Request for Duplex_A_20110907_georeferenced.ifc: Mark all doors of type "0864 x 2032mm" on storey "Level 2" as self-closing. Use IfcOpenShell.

First a look at what the model holds.

```python
import ifcopenshell
import ifcopenshell.util.element

model = ifcopenshell.open("Duplex_A_20110907_georeferenced.ifc")
print(model.schema)
storey = next(s for s in model.by_type("IfcBuildingStorey") if s.Name == "Level 2")
doors = [e for e in ifcopenshell.util.element.get_decomposition(storey) if e.is_a("IfcDoor")]
seen = {}
for e in doors:
    element_type = ifcopenshell.util.element.get_type(e)
    key = (element_type.Name if element_type != e and element_type else None, ifcopenshell.util.element.get_pset(e, "Pset_DoorCommon", "SelfClosing"))
    seen[key] = seen.get(key, 0) + 1
for (name, value), count in sorted(seen.items(), key=str):
    print(count, "x", name, "|", value)
```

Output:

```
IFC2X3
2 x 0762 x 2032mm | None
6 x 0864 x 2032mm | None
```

```python
import ifcopenshell
import ifcopenshell.api.pset
import ifcopenshell.util.element

model = ifcopenshell.open("Duplex_A_20110907_georeferenced.ifc")

storey = next(s for s in model.by_type("IfcBuildingStorey") if s.Name == "Level 2")
doors = [e for e in ifcopenshell.util.element.get_decomposition(storey) if e.is_a("IfcDoor")]

count = 0
for e in doors:
    element_type = ifcopenshell.util.element.get_type(e)
    if element_type in (None, e) or element_type.Name != "0864 x 2032mm":
        continue
    # add_pset returns the element's existing set when there is one.
    pset = ifcopenshell.api.pset.add_pset(model, product=e, name="Pset_DoorCommon")
    ifcopenshell.api.pset.edit_pset(model, pset=pset, properties={"SelfClosing": True})
    count += 1

print(count, "doors updated")

model.write("Duplex_A_20110907_georeferenced_edited.ifc")
```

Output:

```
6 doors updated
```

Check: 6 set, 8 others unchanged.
